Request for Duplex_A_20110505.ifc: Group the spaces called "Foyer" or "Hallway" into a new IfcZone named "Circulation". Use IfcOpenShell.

First a look at what the model holds.

```python
import ifcopenshell

model = ifcopenshell.open("Duplex_A_20110505.ifc")
print(model.schema)
seen = {}
for space in model.by_type("IfcSpace"):
    seen[space.LongName] = seen.get(space.LongName, 0) + 1
for name, count in sorted(seen.items(), key=str):
    print(count, "x", name)
print("zones:", [z.Name for z in model.by_type("IfcZone")][:20])
```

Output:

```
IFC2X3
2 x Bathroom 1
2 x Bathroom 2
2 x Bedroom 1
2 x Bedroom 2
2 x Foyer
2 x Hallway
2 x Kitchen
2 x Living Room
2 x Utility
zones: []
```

```python
import ifcopenshell
import ifcopenshell.api.group
import ifcopenshell.api.root

model = ifcopenshell.open("Duplex_A_20110505.ifc")

names = {"Foyer", "Hallway"}
spaces = [s for s in model.by_type("IfcSpace") if s.LongName in names]

zone = ifcopenshell.api.root.create_entity(model, ifc_class="IfcZone", name="Circulation")
ifcopenshell.api.group.assign_group(model, products=spaces, group=zone)
print(len(spaces), "spaces in", zone.Name)

model.write("Duplex_A_20110505_rev.ifc")
```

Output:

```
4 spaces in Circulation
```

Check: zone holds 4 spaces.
